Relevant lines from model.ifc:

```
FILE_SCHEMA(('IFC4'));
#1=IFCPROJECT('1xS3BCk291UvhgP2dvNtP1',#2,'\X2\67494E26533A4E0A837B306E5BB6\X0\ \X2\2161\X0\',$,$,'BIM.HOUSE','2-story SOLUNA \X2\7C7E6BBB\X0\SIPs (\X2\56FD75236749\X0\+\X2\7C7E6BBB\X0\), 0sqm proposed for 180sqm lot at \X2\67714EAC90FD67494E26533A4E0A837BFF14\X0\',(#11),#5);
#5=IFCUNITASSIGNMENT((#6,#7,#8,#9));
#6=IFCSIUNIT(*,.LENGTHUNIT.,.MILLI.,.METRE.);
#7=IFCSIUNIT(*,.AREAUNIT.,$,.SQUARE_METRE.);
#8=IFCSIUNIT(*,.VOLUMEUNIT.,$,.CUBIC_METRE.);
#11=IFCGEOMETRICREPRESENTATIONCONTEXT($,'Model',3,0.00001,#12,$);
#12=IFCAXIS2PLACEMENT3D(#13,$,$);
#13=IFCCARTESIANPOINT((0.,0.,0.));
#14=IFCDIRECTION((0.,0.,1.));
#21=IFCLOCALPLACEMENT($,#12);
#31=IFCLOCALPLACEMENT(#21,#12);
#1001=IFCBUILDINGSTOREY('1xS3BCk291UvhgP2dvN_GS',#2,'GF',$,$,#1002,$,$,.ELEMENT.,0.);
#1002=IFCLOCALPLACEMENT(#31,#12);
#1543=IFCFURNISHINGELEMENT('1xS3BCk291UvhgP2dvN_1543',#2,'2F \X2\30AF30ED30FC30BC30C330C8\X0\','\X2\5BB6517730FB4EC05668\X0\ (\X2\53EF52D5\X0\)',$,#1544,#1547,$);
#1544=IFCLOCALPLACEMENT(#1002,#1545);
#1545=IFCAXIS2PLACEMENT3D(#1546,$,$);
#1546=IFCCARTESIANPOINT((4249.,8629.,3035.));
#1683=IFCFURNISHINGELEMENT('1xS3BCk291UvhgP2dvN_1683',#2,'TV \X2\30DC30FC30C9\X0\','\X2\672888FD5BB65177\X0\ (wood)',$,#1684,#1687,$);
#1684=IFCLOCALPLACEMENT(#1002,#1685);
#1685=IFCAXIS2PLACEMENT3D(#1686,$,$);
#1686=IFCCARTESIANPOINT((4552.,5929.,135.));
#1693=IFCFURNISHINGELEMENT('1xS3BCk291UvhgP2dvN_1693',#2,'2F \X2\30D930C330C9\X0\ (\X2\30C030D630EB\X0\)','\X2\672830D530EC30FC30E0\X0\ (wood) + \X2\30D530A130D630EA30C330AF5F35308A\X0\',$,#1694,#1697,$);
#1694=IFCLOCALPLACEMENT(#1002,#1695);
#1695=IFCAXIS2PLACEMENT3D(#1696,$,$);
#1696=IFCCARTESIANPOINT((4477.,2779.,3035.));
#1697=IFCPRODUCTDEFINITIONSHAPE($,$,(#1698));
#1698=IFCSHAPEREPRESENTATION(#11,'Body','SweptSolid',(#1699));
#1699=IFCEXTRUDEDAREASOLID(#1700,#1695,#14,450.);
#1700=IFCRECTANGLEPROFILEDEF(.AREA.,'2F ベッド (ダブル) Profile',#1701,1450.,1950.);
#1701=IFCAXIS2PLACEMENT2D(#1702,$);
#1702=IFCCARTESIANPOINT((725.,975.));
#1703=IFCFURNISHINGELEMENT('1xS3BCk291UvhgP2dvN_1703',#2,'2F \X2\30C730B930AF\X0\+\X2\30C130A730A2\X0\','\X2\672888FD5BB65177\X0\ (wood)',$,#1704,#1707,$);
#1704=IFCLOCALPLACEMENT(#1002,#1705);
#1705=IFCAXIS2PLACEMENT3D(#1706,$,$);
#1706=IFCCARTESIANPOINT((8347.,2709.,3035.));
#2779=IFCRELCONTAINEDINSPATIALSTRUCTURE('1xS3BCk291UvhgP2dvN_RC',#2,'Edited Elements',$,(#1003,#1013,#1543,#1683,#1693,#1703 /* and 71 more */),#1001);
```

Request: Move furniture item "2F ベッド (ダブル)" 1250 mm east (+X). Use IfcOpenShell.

```python
import ifcopenshell
import ifcopenshell.api.geometry
import ifcopenshell.util.placement
import ifcopenshell.util.unit

model = ifcopenshell.open("model.ifc")
unit_scale = ifcopenshell.util.unit.calculate_unit_scale(model)

item = model.by_id(1693)
matrix = ifcopenshell.util.placement.get_local_placement(item.ObjectPlacement)
matrix[0, 3] += 1.25 / unit_scale
ifcopenshell.api.geometry.edit_object_placement(model, product=item, matrix=matrix, is_si=False)

print(ifcopenshell.util.placement.get_local_placement(item.ObjectPlacement).round(3) + 0.0)

model.write("model_v2.ifc")
```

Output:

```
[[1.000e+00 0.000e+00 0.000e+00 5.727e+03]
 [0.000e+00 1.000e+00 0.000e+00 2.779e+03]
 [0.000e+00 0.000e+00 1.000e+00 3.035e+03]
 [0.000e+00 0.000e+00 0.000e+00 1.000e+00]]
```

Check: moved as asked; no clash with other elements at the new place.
